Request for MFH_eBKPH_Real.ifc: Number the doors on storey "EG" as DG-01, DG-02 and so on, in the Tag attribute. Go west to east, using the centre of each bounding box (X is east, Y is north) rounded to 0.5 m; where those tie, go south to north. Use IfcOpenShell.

First a look at what the model holds.

```python
import ifcopenshell
import ifcopenshell.util.element
import ifcopenshell.util.placement

model = ifcopenshell.open("MFH_eBKPH_Real.ifc")
print(model.schema)
storey = next(s for s in model.by_type("IfcBuildingStorey") if s.Name == "EG")
doors = [e for e in ifcopenshell.util.element.get_decomposition(storey) if e.is_a("IfcDoor")]
for e in sorted(doors, key=lambda e: e.id()):
    origin = ifcopenshell.util.placement.get_local_placement(e.ObjectPlacement)[:3, 3]
    print(e.id(), e.Tag, e.Name, origin.round(2) + 0.0, sep=" | ")
```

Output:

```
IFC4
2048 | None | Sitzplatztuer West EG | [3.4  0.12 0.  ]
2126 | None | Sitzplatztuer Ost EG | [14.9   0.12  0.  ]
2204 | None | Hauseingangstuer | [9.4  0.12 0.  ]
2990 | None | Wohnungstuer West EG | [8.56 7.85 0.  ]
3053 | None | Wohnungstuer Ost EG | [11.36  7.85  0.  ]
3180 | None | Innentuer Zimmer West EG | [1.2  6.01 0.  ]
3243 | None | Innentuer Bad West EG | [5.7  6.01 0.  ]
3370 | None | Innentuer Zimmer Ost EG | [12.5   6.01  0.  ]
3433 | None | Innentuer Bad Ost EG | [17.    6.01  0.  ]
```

```python
import ifcopenshell
import ifcopenshell.geom
import ifcopenshell.util.element
import ifcopenshell.util.shape

model = ifcopenshell.open("MFH_eBKPH_Real.ifc")
settings = ifcopenshell.geom.settings()
settings.set("use-world-coords", True)


def centre(element):
    shape = ifcopenshell.geom.create_shape(settings, element)
    return ifcopenshell.util.shape.get_bbox_centroid(shape.geometry)


storey = next(s for s in model.by_type("IfcBuildingStorey") if s.Name == "EG")
doors = [e for e in ifcopenshell.util.element.get_decomposition(storey) if e.is_a("IfcDoor")]

# Insertion points can sit at a corner or the storey origin, so sort by the geometry (in metres).
centres = {e: centre(e) for e in doors}
doors.sort(key=lambda e: (round(centres[e][0] / 0.5), centres[e][1]))

for i, e in enumerate(doors, start=1):
    number = f"DG-{i:02d}"
    e.Tag = number
    print(e.id(), number)

model.write("MFH_eBKPH_Real_rev.ifc")
```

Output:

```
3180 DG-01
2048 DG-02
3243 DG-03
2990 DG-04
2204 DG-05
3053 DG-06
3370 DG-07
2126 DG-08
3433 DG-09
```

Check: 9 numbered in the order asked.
